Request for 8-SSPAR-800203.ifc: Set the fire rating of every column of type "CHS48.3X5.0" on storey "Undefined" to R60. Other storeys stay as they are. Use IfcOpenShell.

First a look at what the model holds.

```python
import ifcopenshell
import ifcopenshell.util.element

model = ifcopenshell.open("8-SSPAR-800203.ifc")
print(model.schema)
storey = next(s for s in model.by_type("IfcBuildingStorey") if s.Name == "Undefined")
columns = [e for e in ifcopenshell.util.element.get_decomposition(storey) if e.is_a("IfcColumn")]
seen = {}
for e in columns:
    element_type = ifcopenshell.util.element.get_type(e)
    key = (element_type.Name if element_type != e and element_type else None, ifcopenshell.util.element.get_pset(e, "Pset_ColumnCommon", "FireRating"))
    seen[key] = seen.get(key, 0) + 1
for (name, value), count in sorted(seen.items(), key=str):
    print(count, "x", name, "|", value)
```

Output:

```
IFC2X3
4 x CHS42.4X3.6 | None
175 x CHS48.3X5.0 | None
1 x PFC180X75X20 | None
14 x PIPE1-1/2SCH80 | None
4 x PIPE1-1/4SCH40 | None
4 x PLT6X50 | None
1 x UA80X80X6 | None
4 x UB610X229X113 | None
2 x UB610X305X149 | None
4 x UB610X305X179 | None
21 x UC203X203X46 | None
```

```python
import ifcopenshell
import ifcopenshell.api.pset
import ifcopenshell.util.element

model = ifcopenshell.open("8-SSPAR-800203.ifc")

storey = next(s for s in model.by_type("IfcBuildingStorey") if s.Name == "Undefined")
columns = [e for e in ifcopenshell.util.element.get_decomposition(storey) if e.is_a("IfcColumn")]

count = 0
for e in columns:
    element_type = ifcopenshell.util.element.get_type(e)
    if element_type in (None, e) or element_type.Name != "CHS48.3X5.0":
        continue
    # add_pset returns the element's existing set when there is one.
    pset = ifcopenshell.api.pset.add_pset(model, product=e, name="Pset_ColumnCommon")
    ifcopenshell.api.pset.edit_pset(model, pset=pset, properties={"FireRating": "R60"})
    count += 1

print(count, "columns updated")

model.write("8-SSPAR-800203_rev.ifc")
```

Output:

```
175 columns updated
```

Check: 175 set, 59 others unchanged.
